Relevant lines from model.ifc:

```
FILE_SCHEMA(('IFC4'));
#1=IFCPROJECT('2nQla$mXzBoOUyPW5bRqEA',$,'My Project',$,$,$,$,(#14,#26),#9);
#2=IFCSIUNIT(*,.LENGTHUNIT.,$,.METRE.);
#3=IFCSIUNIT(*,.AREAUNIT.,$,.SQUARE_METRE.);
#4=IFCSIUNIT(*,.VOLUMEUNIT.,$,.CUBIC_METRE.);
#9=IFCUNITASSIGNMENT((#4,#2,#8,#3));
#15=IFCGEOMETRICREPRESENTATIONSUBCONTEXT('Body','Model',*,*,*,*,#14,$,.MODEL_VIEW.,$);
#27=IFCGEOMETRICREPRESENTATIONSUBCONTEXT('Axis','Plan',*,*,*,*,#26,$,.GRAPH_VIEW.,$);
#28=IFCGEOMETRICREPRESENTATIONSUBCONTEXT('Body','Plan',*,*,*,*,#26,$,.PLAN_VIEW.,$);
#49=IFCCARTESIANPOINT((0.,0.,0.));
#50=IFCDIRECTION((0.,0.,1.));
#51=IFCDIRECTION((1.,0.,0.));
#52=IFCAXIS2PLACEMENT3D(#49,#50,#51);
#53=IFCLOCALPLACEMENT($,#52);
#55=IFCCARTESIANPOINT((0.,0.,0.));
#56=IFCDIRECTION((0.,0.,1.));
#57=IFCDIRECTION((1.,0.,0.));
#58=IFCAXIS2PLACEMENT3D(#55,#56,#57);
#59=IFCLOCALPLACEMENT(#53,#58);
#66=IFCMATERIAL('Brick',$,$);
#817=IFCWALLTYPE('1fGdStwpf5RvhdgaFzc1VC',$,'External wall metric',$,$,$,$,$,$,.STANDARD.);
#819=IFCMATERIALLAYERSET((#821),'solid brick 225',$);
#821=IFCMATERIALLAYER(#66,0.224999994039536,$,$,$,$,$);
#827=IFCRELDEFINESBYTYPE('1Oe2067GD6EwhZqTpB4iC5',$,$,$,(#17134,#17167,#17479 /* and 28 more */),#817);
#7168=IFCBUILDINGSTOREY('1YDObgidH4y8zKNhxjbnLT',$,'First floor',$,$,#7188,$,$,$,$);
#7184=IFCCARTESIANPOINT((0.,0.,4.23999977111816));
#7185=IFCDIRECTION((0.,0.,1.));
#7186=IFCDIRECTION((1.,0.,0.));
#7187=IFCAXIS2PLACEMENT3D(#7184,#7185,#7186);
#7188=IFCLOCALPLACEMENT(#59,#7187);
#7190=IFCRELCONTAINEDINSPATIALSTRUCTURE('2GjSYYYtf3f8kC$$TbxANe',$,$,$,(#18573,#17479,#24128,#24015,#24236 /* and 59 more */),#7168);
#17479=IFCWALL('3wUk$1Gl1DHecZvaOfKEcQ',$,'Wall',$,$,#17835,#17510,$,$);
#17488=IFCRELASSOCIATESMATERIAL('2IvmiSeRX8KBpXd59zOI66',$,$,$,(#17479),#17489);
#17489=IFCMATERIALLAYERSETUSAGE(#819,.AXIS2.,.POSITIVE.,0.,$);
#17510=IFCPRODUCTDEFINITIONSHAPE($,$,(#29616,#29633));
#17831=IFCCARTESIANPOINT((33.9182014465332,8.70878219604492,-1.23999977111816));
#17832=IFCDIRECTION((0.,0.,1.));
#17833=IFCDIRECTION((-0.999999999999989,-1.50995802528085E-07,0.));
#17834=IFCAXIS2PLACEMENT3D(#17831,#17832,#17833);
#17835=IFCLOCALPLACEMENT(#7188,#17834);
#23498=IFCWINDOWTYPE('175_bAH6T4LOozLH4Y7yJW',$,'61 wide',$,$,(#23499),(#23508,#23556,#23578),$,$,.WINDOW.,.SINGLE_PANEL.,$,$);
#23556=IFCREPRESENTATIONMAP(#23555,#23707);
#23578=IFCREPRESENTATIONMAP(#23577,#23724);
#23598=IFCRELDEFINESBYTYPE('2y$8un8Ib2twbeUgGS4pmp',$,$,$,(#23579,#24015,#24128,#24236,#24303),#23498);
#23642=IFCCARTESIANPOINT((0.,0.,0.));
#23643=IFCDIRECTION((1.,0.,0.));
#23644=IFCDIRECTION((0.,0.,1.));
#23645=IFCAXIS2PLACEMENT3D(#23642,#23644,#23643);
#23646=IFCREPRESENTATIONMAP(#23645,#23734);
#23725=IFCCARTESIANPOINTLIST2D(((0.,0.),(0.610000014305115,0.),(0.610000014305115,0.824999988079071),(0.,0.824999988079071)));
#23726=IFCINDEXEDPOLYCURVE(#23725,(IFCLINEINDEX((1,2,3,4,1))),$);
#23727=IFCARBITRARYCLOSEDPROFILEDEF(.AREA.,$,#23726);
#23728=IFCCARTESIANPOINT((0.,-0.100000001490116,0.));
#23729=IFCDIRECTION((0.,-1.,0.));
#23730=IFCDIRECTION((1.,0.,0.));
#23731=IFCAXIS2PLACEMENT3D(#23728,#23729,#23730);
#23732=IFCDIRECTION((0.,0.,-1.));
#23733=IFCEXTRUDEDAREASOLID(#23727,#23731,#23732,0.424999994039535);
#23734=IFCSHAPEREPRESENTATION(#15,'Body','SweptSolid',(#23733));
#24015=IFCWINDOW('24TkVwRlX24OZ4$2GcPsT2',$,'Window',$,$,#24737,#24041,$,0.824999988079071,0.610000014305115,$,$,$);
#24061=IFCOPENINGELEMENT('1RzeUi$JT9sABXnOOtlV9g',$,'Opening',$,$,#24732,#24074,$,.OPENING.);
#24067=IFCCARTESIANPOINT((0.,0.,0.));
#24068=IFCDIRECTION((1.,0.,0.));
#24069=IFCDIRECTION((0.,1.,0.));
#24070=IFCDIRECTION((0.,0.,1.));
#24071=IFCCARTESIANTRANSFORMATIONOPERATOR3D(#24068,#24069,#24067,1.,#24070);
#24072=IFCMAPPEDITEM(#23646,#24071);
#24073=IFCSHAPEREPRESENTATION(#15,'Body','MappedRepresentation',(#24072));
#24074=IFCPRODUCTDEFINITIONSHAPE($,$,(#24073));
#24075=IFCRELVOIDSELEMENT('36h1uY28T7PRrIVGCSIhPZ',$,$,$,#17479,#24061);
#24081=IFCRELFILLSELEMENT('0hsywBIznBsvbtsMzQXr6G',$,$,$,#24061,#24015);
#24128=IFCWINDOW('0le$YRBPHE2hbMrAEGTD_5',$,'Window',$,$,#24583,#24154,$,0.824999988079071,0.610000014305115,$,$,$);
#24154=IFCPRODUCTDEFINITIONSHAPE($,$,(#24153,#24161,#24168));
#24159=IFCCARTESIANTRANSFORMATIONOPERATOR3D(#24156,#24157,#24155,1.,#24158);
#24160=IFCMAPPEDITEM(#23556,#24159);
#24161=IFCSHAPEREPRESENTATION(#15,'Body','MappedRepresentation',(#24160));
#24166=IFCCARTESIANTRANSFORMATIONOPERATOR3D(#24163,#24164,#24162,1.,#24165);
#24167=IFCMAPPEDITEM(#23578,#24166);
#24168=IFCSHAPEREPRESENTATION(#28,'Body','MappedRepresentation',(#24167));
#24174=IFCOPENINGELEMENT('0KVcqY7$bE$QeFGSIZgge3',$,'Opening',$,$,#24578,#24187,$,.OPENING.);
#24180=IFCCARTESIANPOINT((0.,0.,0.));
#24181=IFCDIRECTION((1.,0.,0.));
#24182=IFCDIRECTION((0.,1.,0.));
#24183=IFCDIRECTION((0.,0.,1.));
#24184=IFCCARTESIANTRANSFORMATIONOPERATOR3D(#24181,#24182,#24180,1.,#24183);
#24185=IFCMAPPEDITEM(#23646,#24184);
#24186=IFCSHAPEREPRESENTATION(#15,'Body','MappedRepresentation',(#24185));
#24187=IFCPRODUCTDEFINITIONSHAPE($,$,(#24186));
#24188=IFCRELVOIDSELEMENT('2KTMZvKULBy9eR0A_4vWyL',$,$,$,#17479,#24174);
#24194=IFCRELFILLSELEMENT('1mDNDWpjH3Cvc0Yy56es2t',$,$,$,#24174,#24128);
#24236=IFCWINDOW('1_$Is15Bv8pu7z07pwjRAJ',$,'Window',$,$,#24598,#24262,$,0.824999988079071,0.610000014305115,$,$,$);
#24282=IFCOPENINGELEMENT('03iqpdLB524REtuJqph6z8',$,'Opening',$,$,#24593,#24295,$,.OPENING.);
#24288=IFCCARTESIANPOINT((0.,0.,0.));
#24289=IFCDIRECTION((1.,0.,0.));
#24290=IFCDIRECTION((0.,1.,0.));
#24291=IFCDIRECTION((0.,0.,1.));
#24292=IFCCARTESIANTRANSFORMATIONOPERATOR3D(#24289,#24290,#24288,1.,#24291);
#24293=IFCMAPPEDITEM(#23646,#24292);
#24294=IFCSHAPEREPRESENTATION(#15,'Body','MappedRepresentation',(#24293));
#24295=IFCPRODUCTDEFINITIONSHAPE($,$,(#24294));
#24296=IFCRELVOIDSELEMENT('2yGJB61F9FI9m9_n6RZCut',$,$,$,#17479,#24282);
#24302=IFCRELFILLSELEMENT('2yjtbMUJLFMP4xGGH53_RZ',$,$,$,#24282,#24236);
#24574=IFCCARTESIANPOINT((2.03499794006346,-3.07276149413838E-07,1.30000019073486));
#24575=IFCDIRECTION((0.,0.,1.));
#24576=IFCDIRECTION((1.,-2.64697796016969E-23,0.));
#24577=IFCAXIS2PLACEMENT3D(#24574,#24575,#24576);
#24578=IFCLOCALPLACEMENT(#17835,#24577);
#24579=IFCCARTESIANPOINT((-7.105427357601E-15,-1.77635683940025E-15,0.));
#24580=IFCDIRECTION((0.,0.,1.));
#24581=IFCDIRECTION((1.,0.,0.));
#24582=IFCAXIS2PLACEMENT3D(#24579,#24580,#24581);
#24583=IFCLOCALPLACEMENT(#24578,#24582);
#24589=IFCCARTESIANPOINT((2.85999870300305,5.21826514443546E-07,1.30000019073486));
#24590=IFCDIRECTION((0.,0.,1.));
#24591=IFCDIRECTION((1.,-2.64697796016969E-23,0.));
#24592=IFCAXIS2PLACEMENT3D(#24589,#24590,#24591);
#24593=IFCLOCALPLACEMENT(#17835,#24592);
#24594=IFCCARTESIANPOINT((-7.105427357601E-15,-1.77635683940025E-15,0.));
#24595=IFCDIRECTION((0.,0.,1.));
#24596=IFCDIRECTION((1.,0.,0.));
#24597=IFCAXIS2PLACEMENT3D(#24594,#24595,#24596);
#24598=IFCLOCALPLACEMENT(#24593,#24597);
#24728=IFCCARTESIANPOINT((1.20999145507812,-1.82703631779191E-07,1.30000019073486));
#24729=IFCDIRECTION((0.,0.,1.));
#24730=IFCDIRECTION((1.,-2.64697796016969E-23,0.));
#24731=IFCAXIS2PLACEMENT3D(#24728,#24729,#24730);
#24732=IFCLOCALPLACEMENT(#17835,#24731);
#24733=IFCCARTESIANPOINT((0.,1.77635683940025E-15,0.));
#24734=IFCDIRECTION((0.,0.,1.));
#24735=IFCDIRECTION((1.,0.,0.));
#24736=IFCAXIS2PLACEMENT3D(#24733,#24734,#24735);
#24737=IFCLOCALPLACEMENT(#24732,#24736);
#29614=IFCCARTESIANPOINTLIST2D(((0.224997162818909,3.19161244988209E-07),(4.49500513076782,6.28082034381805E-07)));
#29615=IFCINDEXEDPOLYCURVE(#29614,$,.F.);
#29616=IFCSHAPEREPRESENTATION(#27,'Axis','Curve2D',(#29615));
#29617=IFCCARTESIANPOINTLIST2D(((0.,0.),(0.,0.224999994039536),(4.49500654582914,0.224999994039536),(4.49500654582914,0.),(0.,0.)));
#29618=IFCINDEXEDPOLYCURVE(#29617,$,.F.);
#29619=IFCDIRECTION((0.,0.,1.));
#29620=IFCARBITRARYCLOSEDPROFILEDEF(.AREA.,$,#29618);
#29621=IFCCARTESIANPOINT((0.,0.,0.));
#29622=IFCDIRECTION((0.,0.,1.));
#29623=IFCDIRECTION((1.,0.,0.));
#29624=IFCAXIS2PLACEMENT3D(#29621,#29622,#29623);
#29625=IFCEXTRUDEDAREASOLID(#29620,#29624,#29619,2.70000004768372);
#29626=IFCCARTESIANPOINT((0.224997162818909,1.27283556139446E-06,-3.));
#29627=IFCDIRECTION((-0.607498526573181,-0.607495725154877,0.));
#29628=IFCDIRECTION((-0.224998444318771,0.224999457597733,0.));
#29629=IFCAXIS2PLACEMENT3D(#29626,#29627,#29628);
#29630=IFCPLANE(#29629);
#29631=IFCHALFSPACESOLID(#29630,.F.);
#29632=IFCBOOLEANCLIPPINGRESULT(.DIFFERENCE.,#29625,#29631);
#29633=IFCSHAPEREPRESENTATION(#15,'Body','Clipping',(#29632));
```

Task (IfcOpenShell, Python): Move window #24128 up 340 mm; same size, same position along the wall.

```python
import numpy as np
import ifcopenshell
import ifcopenshell.api.geometry
import ifcopenshell.util.placement
import ifcopenshell.util.unit

model = ifcopenshell.open("model.ifc")
unit_scale = ifcopenshell.util.unit.calculate_unit_scale(model)

window = model.by_guid("0le$YRBPHE2hbMrAEGTD_5")
opening = window.FillsVoids[0].RelatingOpeningElement
dz = 0.34

shift = np.array([0.0, 0.0, dz])
# The window is placed relative to its opening, so it follows when the opening moves.
matrix = ifcopenshell.util.placement.get_local_placement(opening.ObjectPlacement)
matrix[:3, 3] += shift
ifcopenshell.api.geometry.edit_object_placement(
    model, product=opening, matrix=matrix, is_si=False, should_transform_children=True
)

print(f"moved by {dz * unit_scale:+.3f} m")

model.write("model-out.ifc")
```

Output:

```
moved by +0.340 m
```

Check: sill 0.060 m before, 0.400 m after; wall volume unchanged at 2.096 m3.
